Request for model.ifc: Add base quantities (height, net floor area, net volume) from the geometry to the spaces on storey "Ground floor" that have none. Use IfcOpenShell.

First a look at what the model holds.

```python
import ifcopenshell
import ifcopenshell.util.element
import ifcopenshell.util.unit

model = ifcopenshell.open("model.ifc")
print(model.schema)
for unit_type in ("LENGTHUNIT", "AREAUNIT", "VOLUMEUNIT"):
    print(unit_type, ifcopenshell.util.unit.calculate_unit_scale(model, unit_type))
storey = next(s for s in model.by_type("IfcBuildingStorey") if s.Name == "Ground floor")
spaces = [e for e in ifcopenshell.util.element.get_decomposition(storey) if e.is_a("IfcSpace")]
for e in sorted(spaces, key=lambda e: e.id()):
    print(e.id(), e.is_a(), e.Name, list(ifcopenshell.util.element.get_psets(e, qtos_only=True)), sep=" | ")
```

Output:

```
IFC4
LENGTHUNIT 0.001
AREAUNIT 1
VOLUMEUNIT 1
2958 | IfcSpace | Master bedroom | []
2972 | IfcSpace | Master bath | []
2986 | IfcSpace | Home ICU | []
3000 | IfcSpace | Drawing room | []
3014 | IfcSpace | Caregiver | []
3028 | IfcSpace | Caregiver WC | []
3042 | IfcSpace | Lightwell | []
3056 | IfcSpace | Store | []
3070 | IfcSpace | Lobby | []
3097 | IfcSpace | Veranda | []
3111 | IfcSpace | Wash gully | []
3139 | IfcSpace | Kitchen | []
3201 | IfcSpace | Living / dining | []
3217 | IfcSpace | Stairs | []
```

```python
import ifcopenshell
import ifcopenshell.api.pset
import ifcopenshell.geom
import ifcopenshell.util.element
import ifcopenshell.util.shape
import ifcopenshell.util.unit

model = ifcopenshell.open("model.ifc")
unit_scale = ifcopenshell.util.unit.calculate_unit_scale(model)
area_scale = ifcopenshell.util.unit.calculate_unit_scale(model, "AREAUNIT")
volume_scale = ifcopenshell.util.unit.calculate_unit_scale(model, "VOLUMEUNIT")
settings = ifcopenshell.geom.settings()

storey = next(s for s in model.by_type("IfcBuildingStorey") if s.Name == "Ground floor")
spaces = [e for e in ifcopenshell.util.element.get_decomposition(storey) if e.is_a("IfcSpace")]

for e in sorted(spaces, key=lambda e: e.id()):
    if ifcopenshell.util.element.get_psets(e, qtos_only=True, should_inherit=False):
        continue
    # Geometry comes back in metres, in the element's own axes.
    shape = ifcopenshell.geom.create_shape(settings, e)
    values = {
        "Height": ifcopenshell.util.shape.get_z(shape.geometry) / unit_scale,
        "NetFloorArea": ifcopenshell.util.shape.get_footprint_area(shape.geometry) / area_scale,
        "NetVolume": ifcopenshell.util.shape.get_volume(shape.geometry) / volume_scale,
    }
    qto = ifcopenshell.api.pset.add_qto(model, product=e, name="Qto_SpaceBaseQuantities")
    ifcopenshell.api.pset.edit_qto(model, qto=qto, properties=values)
    print(e.id(), {k: round(v, 3) for k, v in values.items()})

model.write("model_updated.ifc")
```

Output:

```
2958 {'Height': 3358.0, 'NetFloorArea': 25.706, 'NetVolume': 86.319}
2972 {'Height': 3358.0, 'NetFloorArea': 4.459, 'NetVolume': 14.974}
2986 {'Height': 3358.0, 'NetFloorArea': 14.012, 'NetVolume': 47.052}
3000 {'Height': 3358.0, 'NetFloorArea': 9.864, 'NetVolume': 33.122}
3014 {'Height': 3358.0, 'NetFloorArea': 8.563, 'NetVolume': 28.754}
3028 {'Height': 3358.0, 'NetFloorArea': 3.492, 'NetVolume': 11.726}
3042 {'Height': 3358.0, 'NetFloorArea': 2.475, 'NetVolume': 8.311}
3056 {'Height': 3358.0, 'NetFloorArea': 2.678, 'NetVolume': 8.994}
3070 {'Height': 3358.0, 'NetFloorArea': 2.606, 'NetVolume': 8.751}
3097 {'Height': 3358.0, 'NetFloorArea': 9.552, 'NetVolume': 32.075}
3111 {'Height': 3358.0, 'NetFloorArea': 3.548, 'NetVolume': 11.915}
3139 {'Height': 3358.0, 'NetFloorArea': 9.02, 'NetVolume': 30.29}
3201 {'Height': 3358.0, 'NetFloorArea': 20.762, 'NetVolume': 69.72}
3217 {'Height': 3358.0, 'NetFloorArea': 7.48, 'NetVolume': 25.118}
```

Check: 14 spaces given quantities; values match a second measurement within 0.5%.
